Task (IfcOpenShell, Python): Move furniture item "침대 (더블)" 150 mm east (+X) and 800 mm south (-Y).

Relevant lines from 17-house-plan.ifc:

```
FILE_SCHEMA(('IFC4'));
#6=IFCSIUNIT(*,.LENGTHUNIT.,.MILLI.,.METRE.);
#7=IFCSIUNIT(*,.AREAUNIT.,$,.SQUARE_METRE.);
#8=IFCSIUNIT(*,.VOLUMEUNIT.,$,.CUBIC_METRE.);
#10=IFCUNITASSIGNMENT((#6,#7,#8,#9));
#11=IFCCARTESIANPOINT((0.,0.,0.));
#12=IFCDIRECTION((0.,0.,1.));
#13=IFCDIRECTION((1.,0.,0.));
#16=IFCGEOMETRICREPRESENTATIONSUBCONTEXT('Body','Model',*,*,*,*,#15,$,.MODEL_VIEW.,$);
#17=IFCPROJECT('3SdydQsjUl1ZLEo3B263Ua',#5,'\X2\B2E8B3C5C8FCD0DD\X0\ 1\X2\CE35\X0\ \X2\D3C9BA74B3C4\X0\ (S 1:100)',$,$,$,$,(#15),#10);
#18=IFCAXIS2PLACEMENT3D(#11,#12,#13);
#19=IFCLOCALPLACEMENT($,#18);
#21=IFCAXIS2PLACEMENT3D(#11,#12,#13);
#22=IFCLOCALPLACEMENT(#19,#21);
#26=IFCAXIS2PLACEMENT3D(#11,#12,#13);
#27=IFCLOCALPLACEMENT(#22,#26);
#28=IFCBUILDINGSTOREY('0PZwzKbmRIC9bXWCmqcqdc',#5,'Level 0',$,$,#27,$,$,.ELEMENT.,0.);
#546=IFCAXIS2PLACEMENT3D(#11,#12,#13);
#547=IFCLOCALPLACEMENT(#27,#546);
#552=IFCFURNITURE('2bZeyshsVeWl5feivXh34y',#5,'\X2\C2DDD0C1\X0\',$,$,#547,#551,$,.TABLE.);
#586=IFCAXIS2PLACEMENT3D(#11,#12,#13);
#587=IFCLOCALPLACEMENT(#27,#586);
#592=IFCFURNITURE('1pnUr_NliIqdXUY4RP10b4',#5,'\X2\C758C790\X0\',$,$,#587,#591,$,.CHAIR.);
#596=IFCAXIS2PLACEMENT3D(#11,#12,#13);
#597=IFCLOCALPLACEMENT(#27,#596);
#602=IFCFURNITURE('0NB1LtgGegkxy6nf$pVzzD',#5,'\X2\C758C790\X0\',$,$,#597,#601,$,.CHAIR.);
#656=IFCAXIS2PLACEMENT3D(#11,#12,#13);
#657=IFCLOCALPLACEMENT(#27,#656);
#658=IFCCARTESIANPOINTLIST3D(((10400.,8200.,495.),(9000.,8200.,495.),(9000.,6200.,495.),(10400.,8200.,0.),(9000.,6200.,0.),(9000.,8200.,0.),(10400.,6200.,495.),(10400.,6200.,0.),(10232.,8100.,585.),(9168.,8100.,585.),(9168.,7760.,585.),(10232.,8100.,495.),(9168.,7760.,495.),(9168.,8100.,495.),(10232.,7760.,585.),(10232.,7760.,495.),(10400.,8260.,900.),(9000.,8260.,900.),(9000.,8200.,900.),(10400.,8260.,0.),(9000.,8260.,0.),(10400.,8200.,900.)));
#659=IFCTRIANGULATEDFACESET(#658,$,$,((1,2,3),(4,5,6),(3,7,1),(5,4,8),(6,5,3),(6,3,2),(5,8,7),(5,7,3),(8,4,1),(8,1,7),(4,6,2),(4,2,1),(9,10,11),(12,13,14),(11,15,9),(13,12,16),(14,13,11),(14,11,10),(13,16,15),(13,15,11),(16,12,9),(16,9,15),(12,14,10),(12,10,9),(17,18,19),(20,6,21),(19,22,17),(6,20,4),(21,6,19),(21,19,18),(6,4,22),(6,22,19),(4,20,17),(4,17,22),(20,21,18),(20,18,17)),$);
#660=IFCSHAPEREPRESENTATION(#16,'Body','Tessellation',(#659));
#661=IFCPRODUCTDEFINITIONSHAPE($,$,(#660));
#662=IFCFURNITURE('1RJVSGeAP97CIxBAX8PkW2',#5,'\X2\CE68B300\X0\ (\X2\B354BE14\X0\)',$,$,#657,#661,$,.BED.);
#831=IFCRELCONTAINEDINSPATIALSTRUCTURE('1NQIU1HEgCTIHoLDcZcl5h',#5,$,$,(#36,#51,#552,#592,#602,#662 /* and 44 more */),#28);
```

```python
import ifcopenshell
import ifcopenshell.api.geometry
import ifcopenshell.util.placement
import ifcopenshell.util.unit

model = ifcopenshell.open("17-house-plan.ifc")
unit_scale = ifcopenshell.util.unit.calculate_unit_scale(model)

item = model.by_id(662)
matrix = ifcopenshell.util.placement.get_local_placement(item.ObjectPlacement)
matrix[0, 3] += 0.15 / unit_scale
matrix[1, 3] -= 0.8 / unit_scale
ifcopenshell.api.geometry.edit_object_placement(model, product=item, matrix=matrix, is_si=False)

print(ifcopenshell.util.placement.get_local_placement(item.ObjectPlacement).round(3) + 0.0)

model.write("17-house-plan_updated.ifc")
```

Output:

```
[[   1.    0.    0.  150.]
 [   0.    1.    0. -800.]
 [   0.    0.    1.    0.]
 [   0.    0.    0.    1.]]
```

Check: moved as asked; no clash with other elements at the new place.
